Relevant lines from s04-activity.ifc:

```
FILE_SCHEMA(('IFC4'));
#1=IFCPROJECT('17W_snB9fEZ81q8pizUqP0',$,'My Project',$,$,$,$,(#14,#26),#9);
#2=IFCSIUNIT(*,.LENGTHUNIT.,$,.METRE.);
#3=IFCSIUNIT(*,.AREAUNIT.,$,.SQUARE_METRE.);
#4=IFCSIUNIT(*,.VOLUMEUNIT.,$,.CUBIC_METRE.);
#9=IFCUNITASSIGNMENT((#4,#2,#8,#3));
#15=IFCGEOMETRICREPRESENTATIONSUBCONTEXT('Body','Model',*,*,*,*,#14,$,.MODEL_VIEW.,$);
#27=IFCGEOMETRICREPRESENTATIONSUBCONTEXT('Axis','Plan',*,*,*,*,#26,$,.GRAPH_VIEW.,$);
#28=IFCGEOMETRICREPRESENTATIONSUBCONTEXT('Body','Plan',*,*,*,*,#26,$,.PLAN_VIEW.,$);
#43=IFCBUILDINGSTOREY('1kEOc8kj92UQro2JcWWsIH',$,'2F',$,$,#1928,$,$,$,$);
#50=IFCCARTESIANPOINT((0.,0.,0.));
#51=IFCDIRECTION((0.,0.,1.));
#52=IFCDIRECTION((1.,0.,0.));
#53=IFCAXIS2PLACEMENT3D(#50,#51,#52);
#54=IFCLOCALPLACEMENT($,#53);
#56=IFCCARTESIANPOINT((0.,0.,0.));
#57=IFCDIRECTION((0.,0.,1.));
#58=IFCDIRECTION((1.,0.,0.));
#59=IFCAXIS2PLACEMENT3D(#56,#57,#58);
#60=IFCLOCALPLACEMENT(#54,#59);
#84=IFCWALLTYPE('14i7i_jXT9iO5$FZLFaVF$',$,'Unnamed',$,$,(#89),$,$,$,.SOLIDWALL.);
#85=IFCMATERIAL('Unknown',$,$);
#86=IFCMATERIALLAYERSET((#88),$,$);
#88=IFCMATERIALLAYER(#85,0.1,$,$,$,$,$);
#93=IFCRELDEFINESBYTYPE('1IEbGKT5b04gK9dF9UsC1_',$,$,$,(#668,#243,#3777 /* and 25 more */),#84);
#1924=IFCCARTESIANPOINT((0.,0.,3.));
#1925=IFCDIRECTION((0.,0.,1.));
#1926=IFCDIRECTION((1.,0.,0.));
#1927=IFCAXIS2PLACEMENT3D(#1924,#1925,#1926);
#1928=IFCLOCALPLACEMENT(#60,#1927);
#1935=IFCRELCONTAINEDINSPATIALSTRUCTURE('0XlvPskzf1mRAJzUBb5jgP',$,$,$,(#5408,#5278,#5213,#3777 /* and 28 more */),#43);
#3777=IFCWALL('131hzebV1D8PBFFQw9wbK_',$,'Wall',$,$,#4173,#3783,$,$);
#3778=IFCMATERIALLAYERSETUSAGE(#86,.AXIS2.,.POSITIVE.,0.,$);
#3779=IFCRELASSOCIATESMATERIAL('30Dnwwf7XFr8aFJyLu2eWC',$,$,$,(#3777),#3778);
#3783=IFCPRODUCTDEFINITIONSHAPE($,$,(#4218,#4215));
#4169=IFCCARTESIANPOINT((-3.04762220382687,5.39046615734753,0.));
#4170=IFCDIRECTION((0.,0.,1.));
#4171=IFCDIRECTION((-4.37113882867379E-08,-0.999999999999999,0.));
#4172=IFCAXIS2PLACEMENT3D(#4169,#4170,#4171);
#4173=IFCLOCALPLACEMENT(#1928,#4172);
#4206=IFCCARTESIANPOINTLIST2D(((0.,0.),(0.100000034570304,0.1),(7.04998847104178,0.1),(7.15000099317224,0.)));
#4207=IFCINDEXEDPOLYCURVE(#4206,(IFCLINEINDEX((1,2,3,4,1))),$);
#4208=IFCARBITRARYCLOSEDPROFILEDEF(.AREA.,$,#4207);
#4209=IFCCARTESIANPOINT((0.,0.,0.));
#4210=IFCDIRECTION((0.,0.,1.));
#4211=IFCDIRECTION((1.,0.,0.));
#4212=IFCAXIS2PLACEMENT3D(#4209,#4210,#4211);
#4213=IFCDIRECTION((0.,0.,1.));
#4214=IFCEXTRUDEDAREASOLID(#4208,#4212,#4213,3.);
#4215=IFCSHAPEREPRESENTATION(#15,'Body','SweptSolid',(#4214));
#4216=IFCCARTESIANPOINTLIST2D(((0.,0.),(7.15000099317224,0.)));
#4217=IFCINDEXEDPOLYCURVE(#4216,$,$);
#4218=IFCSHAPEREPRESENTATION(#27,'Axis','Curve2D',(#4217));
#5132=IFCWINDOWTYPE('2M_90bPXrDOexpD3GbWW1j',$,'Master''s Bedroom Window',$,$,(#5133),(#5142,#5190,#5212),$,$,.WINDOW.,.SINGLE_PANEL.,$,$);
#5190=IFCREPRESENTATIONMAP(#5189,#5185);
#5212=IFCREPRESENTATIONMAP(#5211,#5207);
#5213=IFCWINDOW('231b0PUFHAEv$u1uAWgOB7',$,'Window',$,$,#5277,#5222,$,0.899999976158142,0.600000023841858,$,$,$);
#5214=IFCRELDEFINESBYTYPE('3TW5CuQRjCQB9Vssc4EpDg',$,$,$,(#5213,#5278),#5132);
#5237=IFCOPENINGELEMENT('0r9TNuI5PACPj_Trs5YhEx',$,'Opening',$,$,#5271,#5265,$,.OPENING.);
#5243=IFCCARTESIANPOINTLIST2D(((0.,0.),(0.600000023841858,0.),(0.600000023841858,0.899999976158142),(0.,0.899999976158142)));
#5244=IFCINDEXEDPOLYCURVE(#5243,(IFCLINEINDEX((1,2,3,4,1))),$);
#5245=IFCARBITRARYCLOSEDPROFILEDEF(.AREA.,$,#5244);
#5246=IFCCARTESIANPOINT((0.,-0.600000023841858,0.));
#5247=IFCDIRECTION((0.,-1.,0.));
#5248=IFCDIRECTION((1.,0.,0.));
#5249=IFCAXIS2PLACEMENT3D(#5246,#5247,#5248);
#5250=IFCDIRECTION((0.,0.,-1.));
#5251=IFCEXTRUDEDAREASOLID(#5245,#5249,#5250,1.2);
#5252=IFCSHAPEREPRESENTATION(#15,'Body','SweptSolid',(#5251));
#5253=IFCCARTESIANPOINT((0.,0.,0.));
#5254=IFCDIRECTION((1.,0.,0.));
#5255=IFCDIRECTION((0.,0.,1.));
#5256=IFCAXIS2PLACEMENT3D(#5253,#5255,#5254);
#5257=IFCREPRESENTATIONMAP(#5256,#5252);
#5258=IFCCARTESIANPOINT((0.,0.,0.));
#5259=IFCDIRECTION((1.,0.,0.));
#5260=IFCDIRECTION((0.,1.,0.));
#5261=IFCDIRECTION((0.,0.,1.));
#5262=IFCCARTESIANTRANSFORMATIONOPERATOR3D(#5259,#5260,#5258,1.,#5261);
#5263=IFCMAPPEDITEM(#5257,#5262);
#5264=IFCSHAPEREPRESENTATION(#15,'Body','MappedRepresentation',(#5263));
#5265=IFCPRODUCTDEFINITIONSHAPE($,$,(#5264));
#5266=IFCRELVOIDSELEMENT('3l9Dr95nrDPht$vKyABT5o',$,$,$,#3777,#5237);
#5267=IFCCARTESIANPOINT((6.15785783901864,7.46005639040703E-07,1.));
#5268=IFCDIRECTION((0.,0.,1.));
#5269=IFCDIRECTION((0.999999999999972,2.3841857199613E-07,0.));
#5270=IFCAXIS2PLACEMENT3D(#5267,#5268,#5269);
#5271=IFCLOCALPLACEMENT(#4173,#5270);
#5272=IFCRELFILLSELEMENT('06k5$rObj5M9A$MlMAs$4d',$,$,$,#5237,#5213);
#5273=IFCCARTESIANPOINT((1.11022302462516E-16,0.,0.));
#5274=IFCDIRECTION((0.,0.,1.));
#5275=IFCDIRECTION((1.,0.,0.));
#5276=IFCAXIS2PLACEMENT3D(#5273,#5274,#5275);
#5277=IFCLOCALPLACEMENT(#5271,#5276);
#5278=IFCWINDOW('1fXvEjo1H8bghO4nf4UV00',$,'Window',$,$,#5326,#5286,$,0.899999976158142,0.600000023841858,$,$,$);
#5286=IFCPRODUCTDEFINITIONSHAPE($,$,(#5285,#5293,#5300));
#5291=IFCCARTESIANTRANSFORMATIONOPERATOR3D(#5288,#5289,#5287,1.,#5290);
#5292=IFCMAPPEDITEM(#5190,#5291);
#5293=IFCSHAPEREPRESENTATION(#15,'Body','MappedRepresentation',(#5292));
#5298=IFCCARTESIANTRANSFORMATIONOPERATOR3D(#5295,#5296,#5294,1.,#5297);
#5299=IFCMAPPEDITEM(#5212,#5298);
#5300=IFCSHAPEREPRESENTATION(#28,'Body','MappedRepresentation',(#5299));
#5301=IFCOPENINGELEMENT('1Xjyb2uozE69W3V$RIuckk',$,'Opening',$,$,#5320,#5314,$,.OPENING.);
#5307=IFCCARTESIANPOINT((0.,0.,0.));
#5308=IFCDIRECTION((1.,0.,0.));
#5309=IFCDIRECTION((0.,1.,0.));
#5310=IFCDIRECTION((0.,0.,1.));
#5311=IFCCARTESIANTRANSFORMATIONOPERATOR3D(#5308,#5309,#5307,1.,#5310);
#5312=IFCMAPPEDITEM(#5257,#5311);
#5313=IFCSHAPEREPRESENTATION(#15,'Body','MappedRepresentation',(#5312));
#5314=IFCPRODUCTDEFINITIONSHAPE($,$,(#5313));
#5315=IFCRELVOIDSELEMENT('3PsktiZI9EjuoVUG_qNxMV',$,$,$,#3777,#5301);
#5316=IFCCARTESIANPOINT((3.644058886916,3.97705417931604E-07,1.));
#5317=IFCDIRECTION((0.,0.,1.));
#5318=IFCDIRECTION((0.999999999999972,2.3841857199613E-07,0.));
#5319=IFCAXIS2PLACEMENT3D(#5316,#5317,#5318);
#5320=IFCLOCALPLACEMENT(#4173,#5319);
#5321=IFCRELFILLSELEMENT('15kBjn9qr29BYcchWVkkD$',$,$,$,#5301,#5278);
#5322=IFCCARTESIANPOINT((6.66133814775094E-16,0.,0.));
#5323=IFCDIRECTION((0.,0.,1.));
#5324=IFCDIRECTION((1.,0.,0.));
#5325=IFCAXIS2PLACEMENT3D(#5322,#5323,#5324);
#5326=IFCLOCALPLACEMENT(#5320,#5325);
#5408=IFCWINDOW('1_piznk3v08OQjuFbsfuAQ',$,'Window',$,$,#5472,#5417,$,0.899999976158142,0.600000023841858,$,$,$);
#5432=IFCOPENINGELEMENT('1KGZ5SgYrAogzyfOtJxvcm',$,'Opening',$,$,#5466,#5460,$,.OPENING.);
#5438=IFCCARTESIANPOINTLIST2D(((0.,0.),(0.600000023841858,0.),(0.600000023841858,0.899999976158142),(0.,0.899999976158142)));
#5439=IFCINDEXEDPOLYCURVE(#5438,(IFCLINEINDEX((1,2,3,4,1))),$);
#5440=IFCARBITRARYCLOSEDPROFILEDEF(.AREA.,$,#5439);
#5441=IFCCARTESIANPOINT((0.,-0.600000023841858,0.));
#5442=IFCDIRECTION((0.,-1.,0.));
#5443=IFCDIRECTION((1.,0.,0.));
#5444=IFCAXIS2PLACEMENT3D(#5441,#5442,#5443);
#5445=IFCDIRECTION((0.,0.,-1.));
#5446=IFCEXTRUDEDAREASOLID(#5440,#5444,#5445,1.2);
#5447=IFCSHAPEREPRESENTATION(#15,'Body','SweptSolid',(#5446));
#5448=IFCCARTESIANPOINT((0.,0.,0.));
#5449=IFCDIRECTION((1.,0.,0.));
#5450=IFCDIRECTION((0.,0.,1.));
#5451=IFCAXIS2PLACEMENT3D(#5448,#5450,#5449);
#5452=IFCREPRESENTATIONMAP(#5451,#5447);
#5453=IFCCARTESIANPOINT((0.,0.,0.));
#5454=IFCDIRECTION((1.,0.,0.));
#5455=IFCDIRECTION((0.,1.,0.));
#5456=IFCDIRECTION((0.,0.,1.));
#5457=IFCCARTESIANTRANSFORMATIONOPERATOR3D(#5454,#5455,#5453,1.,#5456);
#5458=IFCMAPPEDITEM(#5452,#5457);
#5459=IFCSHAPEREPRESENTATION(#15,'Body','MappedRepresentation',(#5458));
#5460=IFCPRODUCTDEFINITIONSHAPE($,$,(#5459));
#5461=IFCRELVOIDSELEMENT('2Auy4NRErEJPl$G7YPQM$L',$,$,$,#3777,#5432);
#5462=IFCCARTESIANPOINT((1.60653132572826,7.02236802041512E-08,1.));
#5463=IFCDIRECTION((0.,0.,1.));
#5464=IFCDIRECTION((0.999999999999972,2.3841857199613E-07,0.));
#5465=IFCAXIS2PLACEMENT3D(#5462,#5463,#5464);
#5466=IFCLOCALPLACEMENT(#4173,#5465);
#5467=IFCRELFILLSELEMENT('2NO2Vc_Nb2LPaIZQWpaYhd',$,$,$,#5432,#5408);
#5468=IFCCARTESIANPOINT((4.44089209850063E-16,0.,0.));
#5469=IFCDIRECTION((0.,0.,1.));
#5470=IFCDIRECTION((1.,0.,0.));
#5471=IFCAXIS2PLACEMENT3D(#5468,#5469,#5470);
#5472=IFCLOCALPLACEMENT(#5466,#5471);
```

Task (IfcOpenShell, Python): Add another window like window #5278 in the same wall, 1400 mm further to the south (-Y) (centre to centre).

```python
import ifcopenshell
import ifcopenshell.api.feature
import ifcopenshell.api.geometry
import ifcopenshell.api.root
import ifcopenshell.geom
import ifcopenshell.util.element
import ifcopenshell.util.placement
import ifcopenshell.util.shape
import ifcopenshell.util.unit

model = ifcopenshell.open("s04-activity.ifc")
unit_scale = ifcopenshell.util.unit.calculate_unit_scale(model)
settings = ifcopenshell.geom.settings()


def volume(element):
    """Net volume in cubic metres, openings subtracted."""
    shape = ifcopenshell.geom.create_shape(settings, element)
    return ifcopenshell.util.shape.get_volume(shape.geometry)


window = model.by_guid("1fXvEjo1H8bghO4nf4UV00")
opening = window.FillsVoids[0].RelatingOpeningElement
wall = opening.VoidsElements[0].RelatingBuildingElement
before = volume(wall)
shift = ifcopenshell.util.placement.get_local_placement(wall.ObjectPlacement)[:3, 0] * 1.4 / unit_scale

# copy_class copies the void relationship, type, container and properties, but no geometry.
new_opening = ifcopenshell.api.root.copy_class(model, product=opening)
new_opening.Representation = ifcopenshell.util.element.copy_deep(
    model, opening.Representation, exclude=["IfcGeometricRepresentationContext", "IfcRepresentationMap"]
)
new_window = ifcopenshell.api.root.copy_class(model, product=window)
new_window.Representation = ifcopenshell.util.element.copy_deep(
    model, window.Representation, exclude=["IfcGeometricRepresentationContext", "IfcRepresentationMap"]
)
ifcopenshell.api.feature.add_filling(model, opening=new_opening, element=new_window)

for old, new in ((opening, new_opening), (window, new_window)):
    matrix = ifcopenshell.util.placement.get_local_placement(old.ObjectPlacement)
    matrix[:3, 3] += shift
    ifcopenshell.api.geometry.edit_object_placement(model, product=new, matrix=matrix, is_si=False)

after = volume(wall)

print(f"wall volume {before:.3f} -> {after:.3f} m3")

model.write("s04-activity-out.ifc")
```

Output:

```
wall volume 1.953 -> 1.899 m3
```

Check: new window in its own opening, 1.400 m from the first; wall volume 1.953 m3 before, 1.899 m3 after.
